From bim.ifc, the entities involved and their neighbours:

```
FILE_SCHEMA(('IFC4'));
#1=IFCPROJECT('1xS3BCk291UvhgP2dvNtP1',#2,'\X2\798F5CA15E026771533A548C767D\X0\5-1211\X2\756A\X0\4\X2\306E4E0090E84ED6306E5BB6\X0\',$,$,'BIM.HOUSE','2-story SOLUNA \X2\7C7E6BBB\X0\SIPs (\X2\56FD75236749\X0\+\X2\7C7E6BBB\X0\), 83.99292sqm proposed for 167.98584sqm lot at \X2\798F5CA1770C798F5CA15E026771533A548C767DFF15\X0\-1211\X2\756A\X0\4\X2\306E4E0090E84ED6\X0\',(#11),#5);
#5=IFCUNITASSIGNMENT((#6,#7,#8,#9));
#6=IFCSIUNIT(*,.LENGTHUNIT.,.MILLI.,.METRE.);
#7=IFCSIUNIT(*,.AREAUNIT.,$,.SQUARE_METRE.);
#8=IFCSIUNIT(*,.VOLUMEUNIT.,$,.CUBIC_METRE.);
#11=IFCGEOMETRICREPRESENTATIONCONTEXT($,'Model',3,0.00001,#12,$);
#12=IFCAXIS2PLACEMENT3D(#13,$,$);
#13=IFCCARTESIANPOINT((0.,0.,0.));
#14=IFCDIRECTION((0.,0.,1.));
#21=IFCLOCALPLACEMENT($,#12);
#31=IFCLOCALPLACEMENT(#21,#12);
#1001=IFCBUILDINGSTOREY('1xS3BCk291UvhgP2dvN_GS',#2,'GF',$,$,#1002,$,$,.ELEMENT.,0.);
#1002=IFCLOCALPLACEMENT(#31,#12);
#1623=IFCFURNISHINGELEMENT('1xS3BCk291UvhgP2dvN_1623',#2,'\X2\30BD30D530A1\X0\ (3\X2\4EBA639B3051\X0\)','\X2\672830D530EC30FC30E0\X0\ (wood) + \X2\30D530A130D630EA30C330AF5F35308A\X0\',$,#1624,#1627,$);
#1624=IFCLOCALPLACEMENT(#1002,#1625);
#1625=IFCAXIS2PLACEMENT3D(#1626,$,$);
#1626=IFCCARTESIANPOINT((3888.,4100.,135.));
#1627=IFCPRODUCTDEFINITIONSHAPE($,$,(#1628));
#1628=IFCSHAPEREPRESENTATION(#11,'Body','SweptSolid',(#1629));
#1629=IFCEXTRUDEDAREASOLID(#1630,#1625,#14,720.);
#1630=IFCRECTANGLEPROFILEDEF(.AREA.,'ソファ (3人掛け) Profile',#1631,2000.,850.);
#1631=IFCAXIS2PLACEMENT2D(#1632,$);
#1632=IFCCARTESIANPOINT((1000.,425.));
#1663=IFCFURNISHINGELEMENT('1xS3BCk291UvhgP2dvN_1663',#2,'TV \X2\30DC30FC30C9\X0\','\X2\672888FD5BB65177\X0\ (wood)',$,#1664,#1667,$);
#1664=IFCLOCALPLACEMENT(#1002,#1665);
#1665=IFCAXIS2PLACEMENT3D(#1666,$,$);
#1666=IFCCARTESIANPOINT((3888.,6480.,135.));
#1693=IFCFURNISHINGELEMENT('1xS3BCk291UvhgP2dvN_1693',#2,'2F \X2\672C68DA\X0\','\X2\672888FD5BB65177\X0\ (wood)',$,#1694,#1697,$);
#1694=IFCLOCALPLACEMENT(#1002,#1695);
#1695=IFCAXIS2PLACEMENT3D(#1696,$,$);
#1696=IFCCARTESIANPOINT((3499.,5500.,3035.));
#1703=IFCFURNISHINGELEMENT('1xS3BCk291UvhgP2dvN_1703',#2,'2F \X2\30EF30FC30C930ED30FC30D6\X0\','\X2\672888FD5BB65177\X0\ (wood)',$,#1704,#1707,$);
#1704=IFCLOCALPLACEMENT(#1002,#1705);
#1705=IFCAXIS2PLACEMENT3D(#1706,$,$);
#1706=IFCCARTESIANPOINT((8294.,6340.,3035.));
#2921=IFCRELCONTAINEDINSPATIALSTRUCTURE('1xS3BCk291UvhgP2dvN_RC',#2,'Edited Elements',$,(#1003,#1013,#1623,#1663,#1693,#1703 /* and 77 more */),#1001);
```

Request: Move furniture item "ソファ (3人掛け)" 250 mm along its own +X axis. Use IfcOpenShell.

```python
import ifcopenshell
import ifcopenshell.api.geometry
import ifcopenshell.util.placement
import ifcopenshell.util.unit

model = ifcopenshell.open("bim.ifc")
unit_scale = ifcopenshell.util.unit.calculate_unit_scale(model)

item = model.by_guid("1xS3BCk291UvhgP2dvN_1623")
matrix = ifcopenshell.util.placement.get_local_placement(item.ObjectPlacement)
matrix[:3, 3] += matrix[:3, 0] * 0.25 / unit_scale
ifcopenshell.api.geometry.edit_object_placement(model, product=item, matrix=matrix, is_si=False)

print(ifcopenshell.util.placement.get_local_placement(item.ObjectPlacement).round(3) + 0.0)

model.write("bim_v2.ifc")
```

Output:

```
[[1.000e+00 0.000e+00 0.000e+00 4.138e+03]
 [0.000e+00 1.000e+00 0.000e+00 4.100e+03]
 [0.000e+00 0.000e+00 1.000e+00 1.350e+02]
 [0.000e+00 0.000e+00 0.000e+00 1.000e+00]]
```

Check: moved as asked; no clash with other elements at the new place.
